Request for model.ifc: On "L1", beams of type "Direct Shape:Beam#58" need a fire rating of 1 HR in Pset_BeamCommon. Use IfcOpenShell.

First a look at what the model holds.

```python
import ifcopenshell
import ifcopenshell.util.element

model = ifcopenshell.open("model.ifc")
print(model.schema)
storey = next(s for s in model.by_type("IfcBuildingStorey") if s.Name == "L1")
beams = [e for e in ifcopenshell.util.element.get_decomposition(storey) if e.is_a("IfcBeam")]
seen = {}
for e in beams:
    element_type = ifcopenshell.util.element.get_type(e)
    key = (element_type.Name if element_type != e and element_type else None, ifcopenshell.util.element.get_pset(e, "Pset_BeamCommon", "FireRating"))
    seen[key] = seen.get(key, 0) + 1
for (name, value), count in sorted(seen.items(), key=str):
    print(count, "x", name, "|", value)
```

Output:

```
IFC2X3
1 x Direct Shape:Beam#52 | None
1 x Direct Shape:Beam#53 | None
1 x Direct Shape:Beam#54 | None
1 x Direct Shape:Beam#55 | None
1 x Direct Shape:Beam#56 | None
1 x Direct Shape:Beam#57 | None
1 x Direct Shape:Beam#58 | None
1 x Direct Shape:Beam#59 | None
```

```python
import ifcopenshell
import ifcopenshell.api.pset
import ifcopenshell.util.element

model = ifcopenshell.open("model.ifc")

storey = next(s for s in model.by_type("IfcBuildingStorey") if s.Name == "L1")
beams = [e for e in ifcopenshell.util.element.get_decomposition(storey) if e.is_a("IfcBeam")]

count = 0
for e in beams:
    element_type = ifcopenshell.util.element.get_type(e)
    if element_type in (None, e) or element_type.Name != "Direct Shape:Beam#58":
        continue
    # add_pset returns the element's existing set when there is one.
    pset = ifcopenshell.api.pset.add_pset(model, product=e, name="Pset_BeamCommon")
    ifcopenshell.api.pset.edit_pset(model, pset=pset, properties={"FireRating": "1 HR"})
    count += 1

print(count, "beams updated")

model.write("model-out.ifc")
```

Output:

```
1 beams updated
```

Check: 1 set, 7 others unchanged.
